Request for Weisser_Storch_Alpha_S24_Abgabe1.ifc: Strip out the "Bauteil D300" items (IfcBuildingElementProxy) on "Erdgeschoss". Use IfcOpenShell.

First a look at what the model holds.

```python
import ifcopenshell
import ifcopenshell.util.element

model = ifcopenshell.open("Weisser_Storch_Alpha_S24_Abgabe1.ifc")
print(model.schema)
storey = next(s for s in model.by_type("IfcBuildingStorey") if s.Name == "Erdgeschoss")
proxies = [e for e in ifcopenshell.util.element.get_decomposition(storey) if e.is_a("IfcBuildingElementProxy")]
seen = {}
for e in proxies:
    element_type = ifcopenshell.util.element.get_type(e)
    name = element_type.Name if element_type not in (None, e) else None
    seen[name] = seen.get(name, 0) + 1
for name, count in sorted(seen.items(), key=str):
    print(count, "x", name)
```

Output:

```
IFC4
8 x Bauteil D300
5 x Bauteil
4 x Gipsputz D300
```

```python
import ifcopenshell
import ifcopenshell.api.root
import ifcopenshell.util.element

model = ifcopenshell.open("Weisser_Storch_Alpha_S24_Abgabe1.ifc")

storey = next(s for s in model.by_type("IfcBuildingStorey") if s.Name == "Erdgeschoss")
proxies = [e for e in ifcopenshell.util.element.get_decomposition(storey) if e.is_a("IfcBuildingElementProxy")]
targets = [e for e in proxies if (t := ifcopenshell.util.element.get_type(e)) not in (None, e) and t.Name == "Bauteil D300"]

for e in targets:
    ifcopenshell.api.root.remove_product(model, product=e)
print(len(targets), "removed")

model.write("Weisser_Storch_Alpha_S24_Abgabe1_rev.ifc")
```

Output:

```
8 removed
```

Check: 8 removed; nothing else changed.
